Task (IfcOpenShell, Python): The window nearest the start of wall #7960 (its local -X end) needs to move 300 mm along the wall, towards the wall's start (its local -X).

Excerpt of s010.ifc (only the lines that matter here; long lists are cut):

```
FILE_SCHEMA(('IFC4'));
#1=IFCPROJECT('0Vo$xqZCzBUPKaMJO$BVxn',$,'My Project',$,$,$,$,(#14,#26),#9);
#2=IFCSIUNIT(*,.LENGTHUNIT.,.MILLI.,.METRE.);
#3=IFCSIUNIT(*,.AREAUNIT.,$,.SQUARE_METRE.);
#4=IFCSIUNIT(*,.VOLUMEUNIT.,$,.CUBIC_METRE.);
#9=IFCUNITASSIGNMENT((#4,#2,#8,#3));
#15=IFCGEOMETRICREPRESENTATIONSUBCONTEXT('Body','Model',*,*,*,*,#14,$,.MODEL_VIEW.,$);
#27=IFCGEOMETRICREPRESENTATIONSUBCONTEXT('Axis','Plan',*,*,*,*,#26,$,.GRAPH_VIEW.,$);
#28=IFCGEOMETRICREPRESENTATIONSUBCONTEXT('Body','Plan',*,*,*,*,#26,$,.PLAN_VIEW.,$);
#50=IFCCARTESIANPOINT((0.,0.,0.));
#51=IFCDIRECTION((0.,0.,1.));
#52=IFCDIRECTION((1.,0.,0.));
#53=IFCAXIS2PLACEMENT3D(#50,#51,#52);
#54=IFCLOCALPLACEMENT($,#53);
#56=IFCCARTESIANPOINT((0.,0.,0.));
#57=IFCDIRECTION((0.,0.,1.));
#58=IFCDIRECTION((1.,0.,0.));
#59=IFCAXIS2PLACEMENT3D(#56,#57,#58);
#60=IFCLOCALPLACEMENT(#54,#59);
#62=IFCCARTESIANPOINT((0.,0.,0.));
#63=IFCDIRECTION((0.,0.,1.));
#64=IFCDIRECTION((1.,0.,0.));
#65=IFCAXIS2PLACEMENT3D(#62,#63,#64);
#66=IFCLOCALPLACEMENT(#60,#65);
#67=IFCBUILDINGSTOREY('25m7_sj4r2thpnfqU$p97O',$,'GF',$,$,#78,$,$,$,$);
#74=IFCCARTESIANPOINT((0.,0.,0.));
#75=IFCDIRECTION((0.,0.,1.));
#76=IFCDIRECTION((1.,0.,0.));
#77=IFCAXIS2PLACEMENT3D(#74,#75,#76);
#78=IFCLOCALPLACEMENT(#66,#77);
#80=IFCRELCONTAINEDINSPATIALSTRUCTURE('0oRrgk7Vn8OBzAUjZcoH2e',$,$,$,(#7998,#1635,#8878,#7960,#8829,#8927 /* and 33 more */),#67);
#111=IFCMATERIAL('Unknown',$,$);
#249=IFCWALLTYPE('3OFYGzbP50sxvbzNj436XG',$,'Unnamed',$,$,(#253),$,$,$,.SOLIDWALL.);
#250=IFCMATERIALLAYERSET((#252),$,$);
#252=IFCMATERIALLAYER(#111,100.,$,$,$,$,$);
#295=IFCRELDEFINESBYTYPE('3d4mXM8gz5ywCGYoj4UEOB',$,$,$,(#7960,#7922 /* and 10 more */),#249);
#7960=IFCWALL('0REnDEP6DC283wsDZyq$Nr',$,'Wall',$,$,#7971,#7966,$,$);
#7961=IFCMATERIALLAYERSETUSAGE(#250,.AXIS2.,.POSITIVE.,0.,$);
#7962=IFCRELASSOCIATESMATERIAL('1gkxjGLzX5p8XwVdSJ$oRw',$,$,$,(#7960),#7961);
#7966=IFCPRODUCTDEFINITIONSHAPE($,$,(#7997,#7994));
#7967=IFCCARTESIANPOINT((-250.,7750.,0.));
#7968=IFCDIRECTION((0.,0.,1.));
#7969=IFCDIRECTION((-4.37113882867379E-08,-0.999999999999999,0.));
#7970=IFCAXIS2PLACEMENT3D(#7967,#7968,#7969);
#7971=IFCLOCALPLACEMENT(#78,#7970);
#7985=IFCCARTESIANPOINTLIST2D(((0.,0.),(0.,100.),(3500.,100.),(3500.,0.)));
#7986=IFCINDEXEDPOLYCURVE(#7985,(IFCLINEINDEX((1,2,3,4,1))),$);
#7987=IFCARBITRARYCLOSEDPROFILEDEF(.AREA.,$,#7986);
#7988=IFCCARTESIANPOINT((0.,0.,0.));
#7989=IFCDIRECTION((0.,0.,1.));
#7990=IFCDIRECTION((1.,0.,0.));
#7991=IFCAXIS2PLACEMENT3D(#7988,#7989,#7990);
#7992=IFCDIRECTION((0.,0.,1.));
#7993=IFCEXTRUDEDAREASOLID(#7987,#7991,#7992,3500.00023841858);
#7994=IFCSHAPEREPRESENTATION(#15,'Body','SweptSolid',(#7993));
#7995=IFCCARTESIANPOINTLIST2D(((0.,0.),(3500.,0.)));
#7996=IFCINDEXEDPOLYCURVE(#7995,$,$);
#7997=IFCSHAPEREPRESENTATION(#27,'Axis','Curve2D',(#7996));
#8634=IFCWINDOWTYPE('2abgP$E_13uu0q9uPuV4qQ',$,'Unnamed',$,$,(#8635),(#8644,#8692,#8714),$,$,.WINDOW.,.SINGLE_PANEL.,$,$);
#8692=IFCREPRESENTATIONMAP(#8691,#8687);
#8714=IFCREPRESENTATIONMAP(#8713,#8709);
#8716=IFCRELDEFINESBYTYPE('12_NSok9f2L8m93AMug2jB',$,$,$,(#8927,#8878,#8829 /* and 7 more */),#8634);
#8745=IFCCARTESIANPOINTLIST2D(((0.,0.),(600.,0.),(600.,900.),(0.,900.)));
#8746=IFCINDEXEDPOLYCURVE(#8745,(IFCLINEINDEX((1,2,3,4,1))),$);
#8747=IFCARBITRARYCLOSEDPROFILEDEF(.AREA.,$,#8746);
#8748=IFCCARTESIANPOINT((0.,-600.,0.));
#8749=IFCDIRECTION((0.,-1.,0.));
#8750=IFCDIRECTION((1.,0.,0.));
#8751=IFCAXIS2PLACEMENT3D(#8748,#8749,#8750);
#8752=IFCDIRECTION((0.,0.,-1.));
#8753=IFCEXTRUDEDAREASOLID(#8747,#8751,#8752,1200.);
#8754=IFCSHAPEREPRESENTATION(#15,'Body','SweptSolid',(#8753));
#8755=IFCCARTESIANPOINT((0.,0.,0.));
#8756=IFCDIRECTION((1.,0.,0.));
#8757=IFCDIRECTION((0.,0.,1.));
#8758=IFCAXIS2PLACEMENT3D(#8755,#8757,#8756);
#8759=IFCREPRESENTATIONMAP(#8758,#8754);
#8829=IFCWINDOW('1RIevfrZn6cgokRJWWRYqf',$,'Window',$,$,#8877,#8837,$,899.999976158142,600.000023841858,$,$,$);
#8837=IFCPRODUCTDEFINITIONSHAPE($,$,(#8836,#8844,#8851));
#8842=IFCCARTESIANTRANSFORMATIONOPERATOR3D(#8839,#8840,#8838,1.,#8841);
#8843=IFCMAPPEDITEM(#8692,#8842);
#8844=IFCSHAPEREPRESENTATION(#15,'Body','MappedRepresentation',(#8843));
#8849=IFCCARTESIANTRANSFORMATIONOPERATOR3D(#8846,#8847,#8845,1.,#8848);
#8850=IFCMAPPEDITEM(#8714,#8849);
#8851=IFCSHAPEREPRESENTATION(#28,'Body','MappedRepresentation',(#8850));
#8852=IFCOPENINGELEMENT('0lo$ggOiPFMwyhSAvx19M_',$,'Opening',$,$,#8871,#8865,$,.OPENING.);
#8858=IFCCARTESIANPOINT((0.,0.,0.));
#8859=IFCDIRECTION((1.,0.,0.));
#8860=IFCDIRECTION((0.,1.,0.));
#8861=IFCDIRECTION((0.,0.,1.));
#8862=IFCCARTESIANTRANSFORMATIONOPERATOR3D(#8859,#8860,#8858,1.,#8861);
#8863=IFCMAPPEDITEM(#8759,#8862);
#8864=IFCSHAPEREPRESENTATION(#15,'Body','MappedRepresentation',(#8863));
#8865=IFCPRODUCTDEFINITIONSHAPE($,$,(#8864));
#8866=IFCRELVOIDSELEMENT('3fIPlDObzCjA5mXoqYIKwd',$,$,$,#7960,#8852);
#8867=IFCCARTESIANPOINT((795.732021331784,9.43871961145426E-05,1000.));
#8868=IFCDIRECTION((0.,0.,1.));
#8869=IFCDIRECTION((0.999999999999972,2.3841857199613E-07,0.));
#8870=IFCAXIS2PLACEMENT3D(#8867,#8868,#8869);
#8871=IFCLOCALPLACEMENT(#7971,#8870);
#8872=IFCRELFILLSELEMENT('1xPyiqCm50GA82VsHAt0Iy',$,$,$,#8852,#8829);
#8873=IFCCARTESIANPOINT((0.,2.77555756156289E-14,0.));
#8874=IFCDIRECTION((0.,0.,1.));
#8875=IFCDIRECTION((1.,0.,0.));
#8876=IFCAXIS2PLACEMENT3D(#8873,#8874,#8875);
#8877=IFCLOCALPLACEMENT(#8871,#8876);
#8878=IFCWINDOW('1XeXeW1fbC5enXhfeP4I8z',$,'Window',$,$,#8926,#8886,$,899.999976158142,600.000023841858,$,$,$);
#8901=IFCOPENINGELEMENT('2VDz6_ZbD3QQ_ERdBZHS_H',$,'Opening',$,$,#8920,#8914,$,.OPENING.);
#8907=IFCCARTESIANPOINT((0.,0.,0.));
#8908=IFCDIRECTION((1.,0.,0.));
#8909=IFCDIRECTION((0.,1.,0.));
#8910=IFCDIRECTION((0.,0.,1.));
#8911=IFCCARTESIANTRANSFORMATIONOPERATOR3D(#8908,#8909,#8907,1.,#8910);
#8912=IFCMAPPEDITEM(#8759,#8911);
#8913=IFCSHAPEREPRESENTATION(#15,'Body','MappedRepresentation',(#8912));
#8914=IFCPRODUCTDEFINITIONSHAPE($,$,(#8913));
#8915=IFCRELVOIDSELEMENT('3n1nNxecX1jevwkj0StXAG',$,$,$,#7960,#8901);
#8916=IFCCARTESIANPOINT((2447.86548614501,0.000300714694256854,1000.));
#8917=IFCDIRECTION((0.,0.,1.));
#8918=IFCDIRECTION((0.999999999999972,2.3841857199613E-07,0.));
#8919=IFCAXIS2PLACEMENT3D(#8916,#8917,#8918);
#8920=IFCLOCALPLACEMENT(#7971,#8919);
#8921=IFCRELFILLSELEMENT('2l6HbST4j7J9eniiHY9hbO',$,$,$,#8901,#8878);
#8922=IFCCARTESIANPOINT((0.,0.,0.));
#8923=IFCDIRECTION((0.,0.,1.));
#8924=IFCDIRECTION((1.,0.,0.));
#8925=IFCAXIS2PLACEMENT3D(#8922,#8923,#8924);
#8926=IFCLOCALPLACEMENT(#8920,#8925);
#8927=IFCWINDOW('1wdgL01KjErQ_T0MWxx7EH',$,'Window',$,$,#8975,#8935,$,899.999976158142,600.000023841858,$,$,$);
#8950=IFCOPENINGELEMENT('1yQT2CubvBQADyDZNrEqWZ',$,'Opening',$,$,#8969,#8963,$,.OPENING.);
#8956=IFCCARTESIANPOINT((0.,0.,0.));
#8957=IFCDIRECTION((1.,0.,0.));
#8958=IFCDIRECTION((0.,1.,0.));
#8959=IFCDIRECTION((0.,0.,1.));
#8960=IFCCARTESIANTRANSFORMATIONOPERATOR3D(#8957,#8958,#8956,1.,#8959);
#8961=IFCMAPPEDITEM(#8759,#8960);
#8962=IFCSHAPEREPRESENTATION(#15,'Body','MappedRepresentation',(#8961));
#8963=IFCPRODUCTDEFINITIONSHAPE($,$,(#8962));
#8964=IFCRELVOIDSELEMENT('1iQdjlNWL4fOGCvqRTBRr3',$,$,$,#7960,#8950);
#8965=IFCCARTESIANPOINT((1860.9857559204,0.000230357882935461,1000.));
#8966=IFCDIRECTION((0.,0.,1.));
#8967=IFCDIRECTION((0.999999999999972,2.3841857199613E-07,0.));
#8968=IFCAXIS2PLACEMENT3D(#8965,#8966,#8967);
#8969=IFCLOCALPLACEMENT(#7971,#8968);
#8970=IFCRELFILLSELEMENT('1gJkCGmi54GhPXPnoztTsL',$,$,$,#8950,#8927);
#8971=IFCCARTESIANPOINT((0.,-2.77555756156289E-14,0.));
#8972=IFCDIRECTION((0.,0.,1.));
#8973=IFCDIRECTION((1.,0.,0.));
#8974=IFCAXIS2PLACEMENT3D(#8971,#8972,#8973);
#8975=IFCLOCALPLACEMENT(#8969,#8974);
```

```python
import ifcopenshell
import ifcopenshell.api.geometry
import ifcopenshell.util.placement
import ifcopenshell.util.unit

model = ifcopenshell.open("s010.ifc")
unit_scale = ifcopenshell.util.unit.calculate_unit_scale(model)

window = model.by_guid("1RIevfrZn6cgokRJWWRYqf")
opening = window.FillsVoids[0].RelatingOpeningElement
wall = opening.VoidsElements[0].RelatingBuildingElement

wall_matrix = ifcopenshell.util.placement.get_local_placement(wall.ObjectPlacement)
shift = wall_matrix[:3, 0] * -0.3 / unit_scale
before = ifcopenshell.util.placement.get_local_placement(window.ObjectPlacement)[:3, 3].copy()

# The window is placed relative to its opening, so it follows when the opening moves.
matrix = ifcopenshell.util.placement.get_local_placement(opening.ObjectPlacement)
matrix[:3, 3] += shift
ifcopenshell.api.geometry.edit_object_placement(
    model, product=opening, matrix=matrix, is_si=False, should_transform_children=True
)

after = ifcopenshell.util.placement.get_local_placement(window.ObjectPlacement)[:3, 3]
print("window moved by", (after - before).round(3) + 0.0)

model.write("s010-out.ifc")
```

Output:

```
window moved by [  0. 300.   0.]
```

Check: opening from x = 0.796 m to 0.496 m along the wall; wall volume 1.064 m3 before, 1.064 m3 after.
